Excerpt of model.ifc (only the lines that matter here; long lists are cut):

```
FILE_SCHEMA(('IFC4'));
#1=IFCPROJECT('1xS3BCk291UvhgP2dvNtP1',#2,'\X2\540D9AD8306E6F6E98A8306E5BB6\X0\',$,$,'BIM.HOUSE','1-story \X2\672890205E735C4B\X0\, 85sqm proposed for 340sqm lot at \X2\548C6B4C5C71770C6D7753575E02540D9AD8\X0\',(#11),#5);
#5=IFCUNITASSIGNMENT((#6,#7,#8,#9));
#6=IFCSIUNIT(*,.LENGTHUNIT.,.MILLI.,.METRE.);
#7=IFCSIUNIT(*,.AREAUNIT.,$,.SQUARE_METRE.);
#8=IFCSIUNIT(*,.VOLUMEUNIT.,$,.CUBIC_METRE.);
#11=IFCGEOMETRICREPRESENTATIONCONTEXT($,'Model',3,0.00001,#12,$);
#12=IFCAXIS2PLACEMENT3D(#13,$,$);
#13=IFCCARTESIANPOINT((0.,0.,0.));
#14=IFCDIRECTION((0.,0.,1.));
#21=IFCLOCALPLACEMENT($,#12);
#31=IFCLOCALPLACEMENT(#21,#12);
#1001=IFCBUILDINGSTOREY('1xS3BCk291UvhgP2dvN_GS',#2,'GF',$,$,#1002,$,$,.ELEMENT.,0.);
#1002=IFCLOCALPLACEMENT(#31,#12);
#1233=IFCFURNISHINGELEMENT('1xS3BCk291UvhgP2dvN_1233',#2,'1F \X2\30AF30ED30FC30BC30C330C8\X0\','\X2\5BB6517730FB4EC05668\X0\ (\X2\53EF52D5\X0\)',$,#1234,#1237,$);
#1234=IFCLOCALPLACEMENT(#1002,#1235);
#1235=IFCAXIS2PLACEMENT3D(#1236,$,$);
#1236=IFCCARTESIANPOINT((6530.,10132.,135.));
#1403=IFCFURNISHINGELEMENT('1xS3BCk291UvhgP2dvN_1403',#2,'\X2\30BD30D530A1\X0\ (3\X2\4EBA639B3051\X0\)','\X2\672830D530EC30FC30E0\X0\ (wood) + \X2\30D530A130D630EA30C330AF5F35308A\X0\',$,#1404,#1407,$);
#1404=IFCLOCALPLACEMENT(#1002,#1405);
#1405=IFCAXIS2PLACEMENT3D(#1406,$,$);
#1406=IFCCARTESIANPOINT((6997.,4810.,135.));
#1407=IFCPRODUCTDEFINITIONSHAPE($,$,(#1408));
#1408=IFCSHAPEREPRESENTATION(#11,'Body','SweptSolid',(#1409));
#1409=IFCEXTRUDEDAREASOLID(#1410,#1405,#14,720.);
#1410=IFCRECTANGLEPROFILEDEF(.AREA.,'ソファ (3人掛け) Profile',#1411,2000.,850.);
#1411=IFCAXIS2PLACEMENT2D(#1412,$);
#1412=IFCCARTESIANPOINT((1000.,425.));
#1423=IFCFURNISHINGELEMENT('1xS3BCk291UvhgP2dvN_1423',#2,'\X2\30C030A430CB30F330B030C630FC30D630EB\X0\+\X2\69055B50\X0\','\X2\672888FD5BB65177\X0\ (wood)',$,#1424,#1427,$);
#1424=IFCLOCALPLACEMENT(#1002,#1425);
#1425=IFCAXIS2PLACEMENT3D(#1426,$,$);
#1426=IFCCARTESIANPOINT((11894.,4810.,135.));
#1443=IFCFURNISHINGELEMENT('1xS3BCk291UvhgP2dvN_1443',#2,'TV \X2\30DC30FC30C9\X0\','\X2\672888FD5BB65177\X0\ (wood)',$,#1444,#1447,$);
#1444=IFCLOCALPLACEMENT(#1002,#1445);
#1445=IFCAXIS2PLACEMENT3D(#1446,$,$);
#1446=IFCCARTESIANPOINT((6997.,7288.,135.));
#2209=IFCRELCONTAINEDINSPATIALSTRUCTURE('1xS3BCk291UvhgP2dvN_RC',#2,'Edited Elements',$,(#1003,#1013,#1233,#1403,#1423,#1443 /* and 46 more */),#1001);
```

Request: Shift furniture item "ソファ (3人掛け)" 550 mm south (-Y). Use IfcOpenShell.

```python
import ifcopenshell
import ifcopenshell.api.geometry
import ifcopenshell.util.placement

model = ifcopenshell.open("model.ifc")

item = model.by_guid("1xS3BCk291UvhgP2dvN_1403")
matrix = ifcopenshell.util.placement.get_local_placement(item.ObjectPlacement)
matrix[1, 3] -= 550.0
ifcopenshell.api.geometry.edit_object_placement(model, product=item, matrix=matrix, is_si=False)

print(ifcopenshell.util.placement.get_local_placement(item.ObjectPlacement).round(3) + 0.0)

model.write("model_v2.ifc")
```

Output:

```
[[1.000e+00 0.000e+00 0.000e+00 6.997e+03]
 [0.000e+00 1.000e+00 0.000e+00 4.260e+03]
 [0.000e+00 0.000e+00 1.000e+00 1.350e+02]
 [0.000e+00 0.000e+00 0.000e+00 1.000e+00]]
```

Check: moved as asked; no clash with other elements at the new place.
